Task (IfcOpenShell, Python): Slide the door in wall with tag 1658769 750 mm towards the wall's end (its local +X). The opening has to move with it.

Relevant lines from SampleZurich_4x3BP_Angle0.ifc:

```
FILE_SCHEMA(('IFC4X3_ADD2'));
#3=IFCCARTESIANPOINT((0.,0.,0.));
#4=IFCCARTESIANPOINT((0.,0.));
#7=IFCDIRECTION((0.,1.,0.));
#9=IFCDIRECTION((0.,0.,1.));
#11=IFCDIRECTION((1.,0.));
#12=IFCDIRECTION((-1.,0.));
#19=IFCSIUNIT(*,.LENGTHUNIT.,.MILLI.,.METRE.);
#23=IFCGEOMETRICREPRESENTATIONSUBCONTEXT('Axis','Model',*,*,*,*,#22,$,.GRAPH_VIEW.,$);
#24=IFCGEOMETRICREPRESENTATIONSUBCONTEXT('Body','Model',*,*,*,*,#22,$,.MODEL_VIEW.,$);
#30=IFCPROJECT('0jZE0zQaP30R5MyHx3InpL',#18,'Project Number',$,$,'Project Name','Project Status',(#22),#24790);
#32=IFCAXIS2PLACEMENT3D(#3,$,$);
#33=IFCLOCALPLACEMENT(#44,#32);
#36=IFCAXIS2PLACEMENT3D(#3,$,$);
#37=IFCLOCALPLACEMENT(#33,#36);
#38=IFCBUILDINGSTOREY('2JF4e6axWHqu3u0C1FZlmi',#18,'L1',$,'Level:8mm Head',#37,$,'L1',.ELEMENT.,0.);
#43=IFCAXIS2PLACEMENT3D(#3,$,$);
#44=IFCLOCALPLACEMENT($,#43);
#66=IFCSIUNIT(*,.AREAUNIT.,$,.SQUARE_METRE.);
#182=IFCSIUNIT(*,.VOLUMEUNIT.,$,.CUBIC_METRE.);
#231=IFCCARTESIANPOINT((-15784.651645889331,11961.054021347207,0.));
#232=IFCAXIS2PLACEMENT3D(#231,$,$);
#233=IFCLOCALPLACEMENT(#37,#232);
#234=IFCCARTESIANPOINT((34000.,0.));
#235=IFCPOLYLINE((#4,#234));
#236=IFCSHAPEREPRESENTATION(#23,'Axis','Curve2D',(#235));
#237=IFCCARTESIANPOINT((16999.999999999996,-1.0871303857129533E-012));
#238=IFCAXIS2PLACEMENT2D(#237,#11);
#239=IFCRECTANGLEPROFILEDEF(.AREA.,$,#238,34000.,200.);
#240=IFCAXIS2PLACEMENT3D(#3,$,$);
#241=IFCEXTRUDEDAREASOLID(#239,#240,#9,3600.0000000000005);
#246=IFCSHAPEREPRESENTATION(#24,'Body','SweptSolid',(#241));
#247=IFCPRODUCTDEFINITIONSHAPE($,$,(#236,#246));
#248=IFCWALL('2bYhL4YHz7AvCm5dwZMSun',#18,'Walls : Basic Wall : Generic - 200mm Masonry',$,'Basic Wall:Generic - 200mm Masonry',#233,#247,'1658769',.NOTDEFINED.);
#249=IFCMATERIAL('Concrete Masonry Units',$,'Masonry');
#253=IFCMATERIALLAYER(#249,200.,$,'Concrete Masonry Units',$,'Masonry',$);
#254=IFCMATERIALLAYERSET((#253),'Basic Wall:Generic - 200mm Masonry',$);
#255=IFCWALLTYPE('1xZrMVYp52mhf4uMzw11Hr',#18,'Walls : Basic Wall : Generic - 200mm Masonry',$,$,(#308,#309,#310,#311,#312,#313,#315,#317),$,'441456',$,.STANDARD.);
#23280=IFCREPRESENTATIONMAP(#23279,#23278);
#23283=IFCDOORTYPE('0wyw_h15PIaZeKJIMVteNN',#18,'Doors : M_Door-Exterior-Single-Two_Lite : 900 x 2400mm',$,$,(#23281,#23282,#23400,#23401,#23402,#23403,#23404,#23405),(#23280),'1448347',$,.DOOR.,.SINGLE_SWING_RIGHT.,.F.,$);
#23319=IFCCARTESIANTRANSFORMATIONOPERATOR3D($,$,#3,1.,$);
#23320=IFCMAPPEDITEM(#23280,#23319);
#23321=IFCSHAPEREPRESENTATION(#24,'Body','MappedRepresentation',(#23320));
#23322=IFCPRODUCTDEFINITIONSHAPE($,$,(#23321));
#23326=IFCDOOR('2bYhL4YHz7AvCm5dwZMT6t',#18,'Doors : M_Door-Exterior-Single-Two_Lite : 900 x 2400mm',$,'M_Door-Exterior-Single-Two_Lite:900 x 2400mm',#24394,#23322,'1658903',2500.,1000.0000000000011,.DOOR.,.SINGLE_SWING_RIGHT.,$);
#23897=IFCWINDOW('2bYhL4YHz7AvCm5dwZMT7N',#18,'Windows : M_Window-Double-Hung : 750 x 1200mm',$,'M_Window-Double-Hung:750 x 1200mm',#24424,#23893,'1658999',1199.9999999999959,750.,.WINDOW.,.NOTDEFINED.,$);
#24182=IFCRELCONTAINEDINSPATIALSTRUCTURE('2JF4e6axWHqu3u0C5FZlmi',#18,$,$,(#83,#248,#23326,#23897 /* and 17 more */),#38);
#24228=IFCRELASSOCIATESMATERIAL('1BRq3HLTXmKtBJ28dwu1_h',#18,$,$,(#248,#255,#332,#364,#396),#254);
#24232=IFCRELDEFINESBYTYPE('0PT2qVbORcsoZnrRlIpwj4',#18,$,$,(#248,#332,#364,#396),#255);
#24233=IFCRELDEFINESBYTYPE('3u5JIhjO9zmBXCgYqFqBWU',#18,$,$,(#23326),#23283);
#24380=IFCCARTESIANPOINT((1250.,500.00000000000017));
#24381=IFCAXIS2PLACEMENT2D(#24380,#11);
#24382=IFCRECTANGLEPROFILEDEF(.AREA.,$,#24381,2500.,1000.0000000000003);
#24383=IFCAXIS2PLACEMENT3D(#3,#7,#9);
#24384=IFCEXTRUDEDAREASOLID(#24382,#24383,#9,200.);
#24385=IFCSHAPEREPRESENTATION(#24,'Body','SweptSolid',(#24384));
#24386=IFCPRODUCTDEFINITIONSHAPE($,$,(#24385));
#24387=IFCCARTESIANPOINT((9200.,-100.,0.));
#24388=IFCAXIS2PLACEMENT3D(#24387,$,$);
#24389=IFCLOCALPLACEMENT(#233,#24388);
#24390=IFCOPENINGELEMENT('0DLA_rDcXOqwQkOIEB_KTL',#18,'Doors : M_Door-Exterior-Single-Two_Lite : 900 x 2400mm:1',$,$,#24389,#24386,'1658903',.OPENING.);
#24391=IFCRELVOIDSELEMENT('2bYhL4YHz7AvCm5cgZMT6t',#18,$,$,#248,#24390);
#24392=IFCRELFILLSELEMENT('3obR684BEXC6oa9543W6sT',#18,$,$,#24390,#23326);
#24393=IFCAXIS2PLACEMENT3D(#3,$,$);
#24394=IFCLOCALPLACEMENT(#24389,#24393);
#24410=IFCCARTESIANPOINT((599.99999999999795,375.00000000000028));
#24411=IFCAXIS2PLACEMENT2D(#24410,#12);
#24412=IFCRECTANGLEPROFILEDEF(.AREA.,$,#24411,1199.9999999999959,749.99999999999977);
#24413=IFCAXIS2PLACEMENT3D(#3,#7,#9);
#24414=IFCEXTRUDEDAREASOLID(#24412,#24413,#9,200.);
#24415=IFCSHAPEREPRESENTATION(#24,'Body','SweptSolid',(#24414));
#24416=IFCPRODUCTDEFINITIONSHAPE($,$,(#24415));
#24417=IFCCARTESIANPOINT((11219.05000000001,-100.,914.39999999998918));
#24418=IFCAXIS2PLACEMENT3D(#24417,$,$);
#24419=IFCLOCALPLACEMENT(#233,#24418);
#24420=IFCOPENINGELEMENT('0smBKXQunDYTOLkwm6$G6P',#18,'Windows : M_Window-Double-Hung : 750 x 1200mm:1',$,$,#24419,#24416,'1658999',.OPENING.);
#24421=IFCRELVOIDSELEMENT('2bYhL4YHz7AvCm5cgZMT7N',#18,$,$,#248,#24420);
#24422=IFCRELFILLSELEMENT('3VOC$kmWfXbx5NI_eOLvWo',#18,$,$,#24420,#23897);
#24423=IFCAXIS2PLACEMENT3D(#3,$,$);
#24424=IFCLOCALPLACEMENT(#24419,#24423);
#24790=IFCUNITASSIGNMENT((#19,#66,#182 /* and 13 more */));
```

```python
import ifcopenshell
import ifcopenshell.api.geometry
import ifcopenshell.util.placement

model = ifcopenshell.open("SampleZurich_4x3BP_Angle0.ifc")

door = model.by_guid("2bYhL4YHz7AvCm5dwZMT6t")
opening = door.FillsVoids[0].RelatingOpeningElement
wall = opening.VoidsElements[0].RelatingBuildingElement

wall_matrix = ifcopenshell.util.placement.get_local_placement(wall.ObjectPlacement)
shift = wall_matrix[:3, 0] * 750.0
before = ifcopenshell.util.placement.get_local_placement(door.ObjectPlacement)[:3, 3].copy()

# The door is placed relative to its opening, so it follows when the opening moves.
matrix = ifcopenshell.util.placement.get_local_placement(opening.ObjectPlacement)
matrix[:3, 3] += shift
ifcopenshell.api.geometry.edit_object_placement(
    model, product=opening, matrix=matrix, is_si=False, should_transform_children=True
)

after = ifcopenshell.util.placement.get_local_placement(door.ObjectPlacement)[:3, 3]
print("door moved by", (after - before).round(3) + 0.0)

model.write("SampleZurich_4x3BP_Angle0_rev.ifc")
```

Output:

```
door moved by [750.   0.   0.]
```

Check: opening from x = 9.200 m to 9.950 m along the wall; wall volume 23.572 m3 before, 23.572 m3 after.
